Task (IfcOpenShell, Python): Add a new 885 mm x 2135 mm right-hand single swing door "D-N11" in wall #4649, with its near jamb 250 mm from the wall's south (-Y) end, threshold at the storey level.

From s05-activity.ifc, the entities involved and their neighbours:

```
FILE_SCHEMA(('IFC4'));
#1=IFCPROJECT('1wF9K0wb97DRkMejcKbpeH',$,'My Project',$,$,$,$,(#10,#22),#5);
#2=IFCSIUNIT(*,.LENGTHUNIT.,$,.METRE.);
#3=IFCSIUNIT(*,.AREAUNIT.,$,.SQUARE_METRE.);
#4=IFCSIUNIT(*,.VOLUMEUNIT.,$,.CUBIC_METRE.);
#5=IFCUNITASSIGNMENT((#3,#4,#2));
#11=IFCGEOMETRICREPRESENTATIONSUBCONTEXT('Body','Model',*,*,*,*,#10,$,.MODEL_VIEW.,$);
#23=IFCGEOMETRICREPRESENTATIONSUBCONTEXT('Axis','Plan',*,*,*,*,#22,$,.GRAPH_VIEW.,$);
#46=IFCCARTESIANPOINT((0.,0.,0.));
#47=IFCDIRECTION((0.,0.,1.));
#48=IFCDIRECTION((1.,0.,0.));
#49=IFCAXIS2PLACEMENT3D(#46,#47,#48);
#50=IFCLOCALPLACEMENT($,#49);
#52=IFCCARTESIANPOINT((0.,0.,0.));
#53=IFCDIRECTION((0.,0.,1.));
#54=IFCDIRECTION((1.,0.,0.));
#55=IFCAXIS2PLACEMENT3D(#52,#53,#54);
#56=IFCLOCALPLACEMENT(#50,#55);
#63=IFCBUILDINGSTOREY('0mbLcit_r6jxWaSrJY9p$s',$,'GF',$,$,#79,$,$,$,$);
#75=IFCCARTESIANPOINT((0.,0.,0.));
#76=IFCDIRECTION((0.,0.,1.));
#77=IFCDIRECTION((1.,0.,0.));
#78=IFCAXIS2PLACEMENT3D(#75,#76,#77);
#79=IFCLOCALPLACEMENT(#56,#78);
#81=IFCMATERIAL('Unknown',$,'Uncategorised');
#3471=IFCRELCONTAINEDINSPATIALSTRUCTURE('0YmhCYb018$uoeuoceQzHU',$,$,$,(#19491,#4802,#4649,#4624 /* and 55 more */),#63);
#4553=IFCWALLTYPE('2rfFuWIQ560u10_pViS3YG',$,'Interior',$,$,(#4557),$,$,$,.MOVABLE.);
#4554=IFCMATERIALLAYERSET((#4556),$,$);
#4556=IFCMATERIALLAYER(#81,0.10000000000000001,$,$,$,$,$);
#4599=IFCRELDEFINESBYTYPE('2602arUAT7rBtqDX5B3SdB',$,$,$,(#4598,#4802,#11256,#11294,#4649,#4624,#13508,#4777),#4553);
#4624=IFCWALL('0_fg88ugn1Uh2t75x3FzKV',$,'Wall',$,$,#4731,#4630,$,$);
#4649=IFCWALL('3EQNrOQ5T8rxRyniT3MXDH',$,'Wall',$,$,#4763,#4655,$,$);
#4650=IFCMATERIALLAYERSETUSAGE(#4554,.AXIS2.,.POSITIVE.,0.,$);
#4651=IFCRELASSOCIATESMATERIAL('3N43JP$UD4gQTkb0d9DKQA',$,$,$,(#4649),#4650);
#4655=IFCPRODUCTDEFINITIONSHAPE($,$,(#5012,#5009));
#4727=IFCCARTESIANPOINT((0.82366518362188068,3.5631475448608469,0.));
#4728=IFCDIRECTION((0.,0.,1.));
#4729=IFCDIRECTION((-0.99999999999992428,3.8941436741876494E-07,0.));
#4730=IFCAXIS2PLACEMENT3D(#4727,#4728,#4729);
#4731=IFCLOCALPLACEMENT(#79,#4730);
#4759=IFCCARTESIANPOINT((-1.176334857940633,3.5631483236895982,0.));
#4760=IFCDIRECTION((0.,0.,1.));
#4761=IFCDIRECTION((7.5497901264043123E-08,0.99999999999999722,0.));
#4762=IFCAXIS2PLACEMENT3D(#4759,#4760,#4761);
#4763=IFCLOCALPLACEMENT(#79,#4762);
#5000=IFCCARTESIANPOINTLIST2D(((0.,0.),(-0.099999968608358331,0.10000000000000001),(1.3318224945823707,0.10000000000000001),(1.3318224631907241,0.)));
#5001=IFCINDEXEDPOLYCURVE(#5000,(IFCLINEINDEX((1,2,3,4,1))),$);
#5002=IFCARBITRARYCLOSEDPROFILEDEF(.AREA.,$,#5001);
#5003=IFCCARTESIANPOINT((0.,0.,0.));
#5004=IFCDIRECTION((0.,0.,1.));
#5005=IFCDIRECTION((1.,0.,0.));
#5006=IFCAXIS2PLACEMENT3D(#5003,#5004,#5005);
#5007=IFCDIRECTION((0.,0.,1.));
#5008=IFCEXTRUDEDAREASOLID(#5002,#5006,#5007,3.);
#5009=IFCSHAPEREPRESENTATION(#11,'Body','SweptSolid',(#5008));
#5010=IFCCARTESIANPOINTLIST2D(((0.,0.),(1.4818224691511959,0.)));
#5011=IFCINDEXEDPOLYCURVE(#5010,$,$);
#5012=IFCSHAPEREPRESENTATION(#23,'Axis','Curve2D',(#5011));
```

```python
import numpy as np
import ifcopenshell
import ifcopenshell.api.feature
import ifcopenshell.api.geometry
import ifcopenshell.api.root
import ifcopenshell.api.spatial
import ifcopenshell.geom
import ifcopenshell.util.element
import ifcopenshell.util.placement
import ifcopenshell.util.representation
import ifcopenshell.util.shape
import ifcopenshell.util.unit

model = ifcopenshell.open("s05-activity.ifc")
unit_scale = ifcopenshell.util.unit.calculate_unit_scale(model)
settings = ifcopenshell.geom.settings()


def volume(element):
    """Net volume in cubic metres, openings subtracted."""
    shape = ifcopenshell.geom.create_shape(settings, element)
    return ifcopenshell.util.shape.get_volume(shape.geometry)


wall = model.by_guid("3EQNrOQ5T8rxRyniT3MXDH")
storey = ifcopenshell.util.element.get_container(wall, ifc_class="IfcBuildingStorey")
context = ifcopenshell.util.representation.get_context(model, "Model", "Body", "MODEL_VIEW")
before = volume(wall)

width, height, from_end, sill = 0.885, 2.135, 0.25, 0.0  # metres

# The wall runs along its own X axis, and the end named is its -X end.
wall_shape = ifcopenshell.geom.create_shape(settings, wall)
x, y, z = ifcopenshell.util.shape.get_vertices(wall_shape.geometry).T
start = x.min() + from_end
face, thickness = float(y.min()), float(y.max() - y.min())
wall_matrix = ifcopenshell.util.placement.get_local_placement(wall.ObjectPlacement)
level = ifcopenshell.util.placement.get_local_placement(storey.ObjectPlacement)[2, 3]


def in_wall(x, y):
    """Placement at x, y metres in the wall's axes, at sill height."""
    matrix = wall_matrix.copy()
    matrix[:, 3] = wall_matrix @ np.array([x / unit_scale, y / unit_scale, 0.0, 1.0])
    matrix[2, 3] = level + sill / unit_scale
    return matrix


# Opening: a box that overshoots both wall faces by 50 mm.
opening = ifcopenshell.api.root.create_entity(model, ifc_class="IfcOpeningElement", predefined_type="OPENING")
box = ifcopenshell.api.geometry.add_wall_representation(
    model, context=context, length=width, height=height, thickness=thickness + 0.1
)
ifcopenshell.api.geometry.assign_representation(model, product=opening, representation=box)
ifcopenshell.api.geometry.edit_object_placement(model, product=opening, matrix=in_wall(start, face - 0.05), is_si=False)
ifcopenshell.api.feature.add_feature(model, feature=opening, element=wall)

door = ifcopenshell.api.root.create_entity(model, ifc_class="IfcDoor", name="D-N11", predefined_type="DOOR")
door.OverallWidth, door.OverallHeight = width / unit_scale, height / unit_scale
door.OperationType = "SINGLE_SWING_RIGHT"
body = ifcopenshell.api.geometry.add_door_representation(
    model,
    context=context,
    overall_width=door.OverallWidth,
    overall_height=door.OverallHeight,
    operation_type="SINGLE_SWING_RIGHT",
    lining_properties={"LiningDepth": thickness / unit_scale, "ThresholdDepth": thickness / unit_scale},
)
ifcopenshell.api.geometry.assign_representation(model, product=door, representation=body)
ifcopenshell.api.spatial.assign_container(model, products=[door], relating_structure=storey)
ifcopenshell.api.feature.add_filling(model, opening=opening, element=door)

# The lining spans the wall, so the door starts at the wall face.
ifcopenshell.api.geometry.edit_object_placement(model, product=door, matrix=in_wall(start, face), is_si=False)

after = volume(wall)

print(f"wall volume {before:.3f} -> {after:.3f} m3")

model.write("s05-activity_updated.ifc")
```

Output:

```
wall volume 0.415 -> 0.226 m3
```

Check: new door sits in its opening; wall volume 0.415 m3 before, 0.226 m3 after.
